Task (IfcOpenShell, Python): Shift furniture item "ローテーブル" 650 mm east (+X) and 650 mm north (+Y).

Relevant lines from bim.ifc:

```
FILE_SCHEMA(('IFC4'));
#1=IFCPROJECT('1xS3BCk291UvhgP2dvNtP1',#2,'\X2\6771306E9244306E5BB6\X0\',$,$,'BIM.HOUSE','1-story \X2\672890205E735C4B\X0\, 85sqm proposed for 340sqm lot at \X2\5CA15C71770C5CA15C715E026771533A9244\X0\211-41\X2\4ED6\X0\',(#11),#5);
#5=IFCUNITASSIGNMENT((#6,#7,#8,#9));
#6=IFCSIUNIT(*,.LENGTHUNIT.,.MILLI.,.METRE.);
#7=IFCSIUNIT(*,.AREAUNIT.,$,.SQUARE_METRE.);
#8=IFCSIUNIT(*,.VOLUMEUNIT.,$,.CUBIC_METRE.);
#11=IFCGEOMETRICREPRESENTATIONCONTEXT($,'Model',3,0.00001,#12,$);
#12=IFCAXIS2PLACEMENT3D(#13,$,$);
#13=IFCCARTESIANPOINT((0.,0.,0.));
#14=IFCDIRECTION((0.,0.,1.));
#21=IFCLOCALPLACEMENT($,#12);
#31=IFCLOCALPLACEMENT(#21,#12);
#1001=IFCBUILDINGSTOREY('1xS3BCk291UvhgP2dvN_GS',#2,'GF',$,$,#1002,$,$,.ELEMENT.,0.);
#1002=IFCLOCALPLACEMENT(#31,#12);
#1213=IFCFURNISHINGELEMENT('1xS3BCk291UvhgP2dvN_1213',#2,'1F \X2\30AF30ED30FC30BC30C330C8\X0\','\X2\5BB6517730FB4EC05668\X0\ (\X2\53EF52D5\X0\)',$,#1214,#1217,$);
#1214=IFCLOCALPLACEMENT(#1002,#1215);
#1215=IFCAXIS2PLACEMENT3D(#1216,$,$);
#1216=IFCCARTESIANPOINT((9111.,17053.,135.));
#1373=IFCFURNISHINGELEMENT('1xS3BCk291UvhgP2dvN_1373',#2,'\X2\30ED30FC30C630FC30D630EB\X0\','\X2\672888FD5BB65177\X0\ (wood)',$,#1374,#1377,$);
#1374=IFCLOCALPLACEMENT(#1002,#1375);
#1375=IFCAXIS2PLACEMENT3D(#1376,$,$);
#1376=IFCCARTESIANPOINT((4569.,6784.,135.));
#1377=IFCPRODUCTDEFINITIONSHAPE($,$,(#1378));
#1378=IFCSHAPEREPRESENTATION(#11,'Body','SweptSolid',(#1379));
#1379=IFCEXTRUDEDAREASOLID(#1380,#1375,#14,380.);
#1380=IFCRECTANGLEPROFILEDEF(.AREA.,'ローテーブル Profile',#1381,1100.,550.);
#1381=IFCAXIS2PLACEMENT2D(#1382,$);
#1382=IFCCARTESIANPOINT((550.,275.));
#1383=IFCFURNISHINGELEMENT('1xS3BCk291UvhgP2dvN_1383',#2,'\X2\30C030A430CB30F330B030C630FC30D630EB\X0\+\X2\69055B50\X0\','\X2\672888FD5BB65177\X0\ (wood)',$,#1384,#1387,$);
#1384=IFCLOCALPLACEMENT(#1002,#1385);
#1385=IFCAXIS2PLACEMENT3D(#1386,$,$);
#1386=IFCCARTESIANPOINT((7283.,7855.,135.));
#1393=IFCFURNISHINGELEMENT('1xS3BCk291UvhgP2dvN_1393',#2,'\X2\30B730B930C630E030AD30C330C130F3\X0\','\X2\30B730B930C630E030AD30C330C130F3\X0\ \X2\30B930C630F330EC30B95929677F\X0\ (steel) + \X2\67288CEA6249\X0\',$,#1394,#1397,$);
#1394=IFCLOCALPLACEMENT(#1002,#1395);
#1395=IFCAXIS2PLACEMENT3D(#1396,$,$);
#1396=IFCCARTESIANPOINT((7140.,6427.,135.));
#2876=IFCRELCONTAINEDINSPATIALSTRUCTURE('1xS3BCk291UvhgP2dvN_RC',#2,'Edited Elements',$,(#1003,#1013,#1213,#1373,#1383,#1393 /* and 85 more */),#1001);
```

```python
import ifcopenshell
import ifcopenshell.api.geometry
import ifcopenshell.util.placement

model = ifcopenshell.open("bim.ifc")

item = model.by_id(1373)
matrix = ifcopenshell.util.placement.get_local_placement(item.ObjectPlacement)
matrix[0, 3] += 650.0
matrix[1, 3] += 650.0
ifcopenshell.api.geometry.edit_object_placement(model, product=item, matrix=matrix, is_si=False)

print(ifcopenshell.util.placement.get_local_placement(item.ObjectPlacement).round(3) + 0.0)

model.write("bim_edited.ifc")
```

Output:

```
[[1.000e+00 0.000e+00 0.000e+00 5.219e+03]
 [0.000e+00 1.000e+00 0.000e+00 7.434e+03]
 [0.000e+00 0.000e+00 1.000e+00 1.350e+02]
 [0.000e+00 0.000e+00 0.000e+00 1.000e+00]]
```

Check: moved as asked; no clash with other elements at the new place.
